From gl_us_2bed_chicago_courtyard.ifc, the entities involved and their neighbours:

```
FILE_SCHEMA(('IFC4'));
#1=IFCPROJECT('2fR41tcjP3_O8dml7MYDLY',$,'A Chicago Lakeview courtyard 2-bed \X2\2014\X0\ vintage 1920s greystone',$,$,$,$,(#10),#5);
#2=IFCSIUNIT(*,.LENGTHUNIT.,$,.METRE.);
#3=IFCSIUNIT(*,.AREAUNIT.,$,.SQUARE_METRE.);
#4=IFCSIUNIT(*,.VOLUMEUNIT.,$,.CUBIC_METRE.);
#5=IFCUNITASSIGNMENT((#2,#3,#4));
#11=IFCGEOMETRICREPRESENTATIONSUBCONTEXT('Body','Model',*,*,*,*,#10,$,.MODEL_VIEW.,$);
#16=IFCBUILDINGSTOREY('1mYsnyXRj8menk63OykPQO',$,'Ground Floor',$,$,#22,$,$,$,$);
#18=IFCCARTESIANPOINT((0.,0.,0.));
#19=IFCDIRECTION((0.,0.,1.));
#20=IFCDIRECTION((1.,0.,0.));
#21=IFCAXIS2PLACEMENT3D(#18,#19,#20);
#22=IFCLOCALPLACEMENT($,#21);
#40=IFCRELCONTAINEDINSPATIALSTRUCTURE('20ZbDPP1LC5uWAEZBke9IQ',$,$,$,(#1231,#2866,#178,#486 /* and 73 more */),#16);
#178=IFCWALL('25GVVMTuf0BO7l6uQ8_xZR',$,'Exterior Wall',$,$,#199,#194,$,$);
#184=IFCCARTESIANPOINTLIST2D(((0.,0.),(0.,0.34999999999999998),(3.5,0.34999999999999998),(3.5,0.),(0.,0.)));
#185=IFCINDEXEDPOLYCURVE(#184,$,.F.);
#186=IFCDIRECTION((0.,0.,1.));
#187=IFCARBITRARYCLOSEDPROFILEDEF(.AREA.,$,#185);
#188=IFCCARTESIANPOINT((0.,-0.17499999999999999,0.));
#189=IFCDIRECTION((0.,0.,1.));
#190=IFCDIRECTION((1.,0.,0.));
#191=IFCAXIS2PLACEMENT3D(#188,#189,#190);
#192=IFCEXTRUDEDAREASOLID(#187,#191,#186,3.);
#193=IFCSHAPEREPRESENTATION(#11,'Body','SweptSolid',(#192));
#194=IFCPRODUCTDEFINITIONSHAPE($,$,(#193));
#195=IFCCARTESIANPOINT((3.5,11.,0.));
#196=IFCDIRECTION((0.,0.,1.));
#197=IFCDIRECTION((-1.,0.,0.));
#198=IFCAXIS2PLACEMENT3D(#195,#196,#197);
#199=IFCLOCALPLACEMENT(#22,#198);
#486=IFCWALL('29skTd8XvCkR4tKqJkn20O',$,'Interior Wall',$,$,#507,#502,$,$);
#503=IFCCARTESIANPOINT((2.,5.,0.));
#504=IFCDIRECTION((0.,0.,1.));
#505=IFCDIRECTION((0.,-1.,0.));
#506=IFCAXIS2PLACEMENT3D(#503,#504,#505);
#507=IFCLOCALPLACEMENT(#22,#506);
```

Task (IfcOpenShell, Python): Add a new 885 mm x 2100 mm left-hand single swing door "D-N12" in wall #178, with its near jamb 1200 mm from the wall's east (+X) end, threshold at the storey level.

```python
import numpy as np
import ifcopenshell
import ifcopenshell.api.feature
import ifcopenshell.api.geometry
import ifcopenshell.api.root
import ifcopenshell.api.spatial
import ifcopenshell.geom
import ifcopenshell.util.element
import ifcopenshell.util.placement
import ifcopenshell.util.representation
import ifcopenshell.util.shape
import ifcopenshell.util.unit

model = ifcopenshell.open("gl_us_2bed_chicago_courtyard.ifc")
unit_scale = ifcopenshell.util.unit.calculate_unit_scale(model)
settings = ifcopenshell.geom.settings()


def volume(element):
    """Net volume in cubic metres, openings subtracted."""
    shape = ifcopenshell.geom.create_shape(settings, element)
    return ifcopenshell.util.shape.get_volume(shape.geometry)


wall = model.by_id(178)
storey = ifcopenshell.util.element.get_container(wall, ifc_class="IfcBuildingStorey")
context = ifcopenshell.util.representation.get_context(model, "Model", "Body", "MODEL_VIEW")
before = volume(wall)

width, height, from_end, sill = 0.885, 2.1, 1.2, 0.0  # metres

# The wall runs along its own X axis, and the end named is its -X end.
wall_shape = ifcopenshell.geom.create_shape(settings, wall)
x, y, z = ifcopenshell.util.shape.get_vertices(wall_shape.geometry).T
start = x.min() + from_end
face, thickness = float(y.min()), float(y.max() - y.min())
wall_matrix = ifcopenshell.util.placement.get_local_placement(wall.ObjectPlacement)
level = ifcopenshell.util.placement.get_local_placement(storey.ObjectPlacement)[2, 3]


def in_wall(x, y):
    """Placement at x, y metres in the wall's axes, at sill height."""
    matrix = wall_matrix.copy()
    matrix[:, 3] = wall_matrix @ np.array([x / unit_scale, y / unit_scale, 0.0, 1.0])
    matrix[2, 3] = level + sill / unit_scale
    return matrix


# Opening: a box that overshoots both wall faces by 50 mm.
opening = ifcopenshell.api.root.create_entity(model, ifc_class="IfcOpeningElement", predefined_type="OPENING")
box = ifcopenshell.api.geometry.add_wall_representation(
    model, context=context, length=width, height=height, thickness=thickness + 0.1
)
ifcopenshell.api.geometry.assign_representation(model, product=opening, representation=box)
ifcopenshell.api.geometry.edit_object_placement(model, product=opening, matrix=in_wall(start, face - 0.05), is_si=False)
ifcopenshell.api.feature.add_feature(model, feature=opening, element=wall)

door = ifcopenshell.api.root.create_entity(model, ifc_class="IfcDoor", name="D-N12", predefined_type="DOOR")
door.OverallWidth, door.OverallHeight = width / unit_scale, height / unit_scale
door.OperationType = "SINGLE_SWING_LEFT"
body = ifcopenshell.api.geometry.add_door_representation(
    model,
    context=context,
    overall_width=door.OverallWidth,
    overall_height=door.OverallHeight,
    operation_type="SINGLE_SWING_LEFT",
    lining_properties={"LiningDepth": thickness / unit_scale, "ThresholdDepth": thickness / unit_scale},
)
ifcopenshell.api.geometry.assign_representation(model, product=door, representation=body)
ifcopenshell.api.spatial.assign_container(model, products=[door], relating_structure=storey)
ifcopenshell.api.feature.add_filling(model, opening=opening, element=door)

# The lining spans the wall, so the door starts at the wall face.
ifcopenshell.api.geometry.edit_object_placement(model, product=door, matrix=in_wall(start, face), is_si=False)

after = volume(wall)

print(f"wall volume {before:.3f} -> {after:.3f} m3")

model.write("gl_us_2bed_chicago_courtyard_rev.ifc")
```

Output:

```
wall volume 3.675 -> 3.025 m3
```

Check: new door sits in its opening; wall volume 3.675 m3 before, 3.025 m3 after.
